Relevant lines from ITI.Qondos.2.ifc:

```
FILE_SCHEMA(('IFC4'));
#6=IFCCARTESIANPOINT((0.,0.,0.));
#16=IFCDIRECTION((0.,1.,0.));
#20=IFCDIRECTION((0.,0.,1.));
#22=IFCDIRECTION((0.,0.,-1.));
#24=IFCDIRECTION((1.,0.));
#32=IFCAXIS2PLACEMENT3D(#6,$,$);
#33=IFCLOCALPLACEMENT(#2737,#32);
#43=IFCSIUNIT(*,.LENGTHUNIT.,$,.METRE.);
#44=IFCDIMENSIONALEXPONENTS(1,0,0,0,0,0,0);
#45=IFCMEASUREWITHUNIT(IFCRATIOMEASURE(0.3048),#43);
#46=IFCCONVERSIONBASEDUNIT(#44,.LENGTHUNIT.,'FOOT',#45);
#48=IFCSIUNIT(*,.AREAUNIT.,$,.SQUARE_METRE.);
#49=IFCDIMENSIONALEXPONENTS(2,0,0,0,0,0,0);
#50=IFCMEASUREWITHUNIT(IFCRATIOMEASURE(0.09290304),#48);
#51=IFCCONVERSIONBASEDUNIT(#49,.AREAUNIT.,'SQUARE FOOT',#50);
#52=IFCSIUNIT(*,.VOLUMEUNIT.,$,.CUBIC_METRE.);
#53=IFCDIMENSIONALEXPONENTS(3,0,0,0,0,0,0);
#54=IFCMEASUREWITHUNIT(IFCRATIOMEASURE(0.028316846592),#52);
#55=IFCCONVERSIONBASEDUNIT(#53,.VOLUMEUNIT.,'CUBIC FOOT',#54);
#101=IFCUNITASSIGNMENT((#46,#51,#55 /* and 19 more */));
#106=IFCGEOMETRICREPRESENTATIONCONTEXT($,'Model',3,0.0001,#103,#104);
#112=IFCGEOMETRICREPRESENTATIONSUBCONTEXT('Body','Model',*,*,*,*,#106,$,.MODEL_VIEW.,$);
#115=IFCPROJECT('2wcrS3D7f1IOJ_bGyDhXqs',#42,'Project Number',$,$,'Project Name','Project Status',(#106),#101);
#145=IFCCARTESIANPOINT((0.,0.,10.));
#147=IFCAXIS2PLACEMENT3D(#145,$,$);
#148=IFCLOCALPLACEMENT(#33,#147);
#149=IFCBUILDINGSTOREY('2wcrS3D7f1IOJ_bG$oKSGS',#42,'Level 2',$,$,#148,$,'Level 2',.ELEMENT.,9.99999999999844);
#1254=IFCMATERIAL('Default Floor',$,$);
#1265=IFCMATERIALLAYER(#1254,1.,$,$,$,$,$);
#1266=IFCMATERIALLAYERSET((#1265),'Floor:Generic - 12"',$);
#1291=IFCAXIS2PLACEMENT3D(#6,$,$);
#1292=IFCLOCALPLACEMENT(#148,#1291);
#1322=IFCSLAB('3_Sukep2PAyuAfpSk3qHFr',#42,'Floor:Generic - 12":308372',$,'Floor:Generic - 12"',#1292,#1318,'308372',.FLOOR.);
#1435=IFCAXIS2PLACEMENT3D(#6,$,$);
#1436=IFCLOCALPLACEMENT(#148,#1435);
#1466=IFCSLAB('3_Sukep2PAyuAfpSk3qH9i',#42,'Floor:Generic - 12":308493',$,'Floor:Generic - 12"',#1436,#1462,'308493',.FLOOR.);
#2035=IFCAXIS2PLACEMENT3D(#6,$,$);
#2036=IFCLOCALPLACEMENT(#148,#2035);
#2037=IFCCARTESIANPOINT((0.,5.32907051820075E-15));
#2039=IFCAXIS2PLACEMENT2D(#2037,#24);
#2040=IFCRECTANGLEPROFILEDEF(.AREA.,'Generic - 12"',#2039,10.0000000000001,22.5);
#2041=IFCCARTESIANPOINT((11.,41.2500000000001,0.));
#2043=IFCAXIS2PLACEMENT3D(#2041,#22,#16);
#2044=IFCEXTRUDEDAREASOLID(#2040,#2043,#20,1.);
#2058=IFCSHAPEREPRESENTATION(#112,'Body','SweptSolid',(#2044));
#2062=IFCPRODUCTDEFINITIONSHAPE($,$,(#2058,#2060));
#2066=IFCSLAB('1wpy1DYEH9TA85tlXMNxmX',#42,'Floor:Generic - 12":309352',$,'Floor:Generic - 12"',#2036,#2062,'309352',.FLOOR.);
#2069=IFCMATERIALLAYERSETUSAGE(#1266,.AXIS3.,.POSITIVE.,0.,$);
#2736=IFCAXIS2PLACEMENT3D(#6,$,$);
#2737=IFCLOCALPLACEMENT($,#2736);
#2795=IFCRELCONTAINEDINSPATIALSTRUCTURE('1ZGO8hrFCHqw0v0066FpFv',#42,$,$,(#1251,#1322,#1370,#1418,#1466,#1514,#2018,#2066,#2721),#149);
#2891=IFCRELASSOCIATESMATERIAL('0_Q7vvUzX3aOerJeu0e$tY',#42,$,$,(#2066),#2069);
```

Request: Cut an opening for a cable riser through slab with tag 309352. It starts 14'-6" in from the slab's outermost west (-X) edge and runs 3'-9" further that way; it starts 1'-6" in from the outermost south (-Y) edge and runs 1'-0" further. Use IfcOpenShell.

```python
import numpy as np
import ifcopenshell
import ifcopenshell.api.feature
import ifcopenshell.api.geometry
import ifcopenshell.api.root
import ifcopenshell.geom
import ifcopenshell.util.placement
import ifcopenshell.util.representation
import ifcopenshell.util.shape
import ifcopenshell.util.unit

model = ifcopenshell.open("ITI.Qondos.2.ifc")
unit_scale = ifcopenshell.util.unit.calculate_unit_scale(model)
settings = ifcopenshell.geom.settings()


def volume(element):
    """Net volume in cubic metres, openings subtracted."""
    shape = ifcopenshell.geom.create_shape(settings, element)
    return ifcopenshell.util.shape.get_volume(shape.geometry)


slab = model.by_guid("1wpy1DYEH9TA85tlXMNxmX")
before = volume(slab)

# Extent in the slab's own axes, in metres. The edges named are its -X and -Y sides.
slab_shape = ifcopenshell.geom.create_shape(settings, slab)
vertices = ifcopenshell.util.shape.get_vertices(slab_shape.geometry)
x_min, y_min, bottom = vertices.min(axis=0)
top = vertices[:, 2].max()

opening = ifcopenshell.api.root.create_entity(model, ifc_class="IfcOpeningElement", name="Cable riser opening", predefined_type="OPENING")
context = ifcopenshell.util.representation.get_context(model, "Model", "Body", "MODEL_VIEW")
width, depth = 1.143, 0.3048
outline = [(0.0, 0.0), (width, 0.0), (width, depth), (0.0, depth), (0.0, 0.0)]
# Overshoot both faces by 50 mm so the cut is clean.
shape = ifcopenshell.api.geometry.add_slab_representation(
    model, context=context, depth=top - bottom + 0.1, polyline=outline
)
ifcopenshell.api.geometry.assign_representation(model, product=opening, representation=shape)

matrix = ifcopenshell.util.placement.get_local_placement(slab.ObjectPlacement)
matrix[:, 3] = matrix @ np.append(np.array([x_min + 4.4196, y_min + 0.4572, bottom - 0.05]) / unit_scale, 1.0)
ifcopenshell.api.geometry.edit_object_placement(model, product=opening, matrix=matrix, is_si=False)
ifcopenshell.api.feature.add_feature(model, feature=opening, element=slab)

after = volume(slab)

print(f"slab volume {before:.3f} -> {after:.3f} m3")

model.write("ITI.Qondos.2_v2.ifc")
```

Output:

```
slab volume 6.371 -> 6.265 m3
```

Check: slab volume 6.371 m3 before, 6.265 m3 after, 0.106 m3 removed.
